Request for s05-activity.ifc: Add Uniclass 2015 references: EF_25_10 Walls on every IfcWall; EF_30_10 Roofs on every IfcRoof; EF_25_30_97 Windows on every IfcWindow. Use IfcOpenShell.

First a look at what the model holds.

```python
import ifcopenshell

model = ifcopenshell.open("s05-activity.ifc")
print(model.schema)
print("classifications:", [c.Name for c in model.by_type("IfcClassification")])
for ifc_class in ("IfcDoor", "IfcRoof", "IfcStair", "IfcWall", "IfcWindow"):
    print(ifc_class, len(model.by_type(ifc_class)))
```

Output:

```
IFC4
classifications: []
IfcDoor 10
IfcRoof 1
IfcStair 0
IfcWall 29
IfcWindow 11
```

```python
import ifcopenshell
import ifcopenshell.api.classification

model = ifcopenshell.open("s05-activity.ifc")

system = ifcopenshell.api.classification.add_classification(model, classification="Uniclass 2015")

codes = {
    "IfcWall": ("EF_25_10", "Walls"),
    "IfcRoof": ("EF_30_10", "Roofs"),
    "IfcWindow": ("EF_25_30_97", "Windows"),
}
for ifc_class, (code, name) in codes.items():
    products = model.by_type(ifc_class)
    ifcopenshell.api.classification.add_reference(
        model, products=products, classification=system, identification=code, name=name
    )
    print(code, len(products))

model.write("s05-activity_v2.ifc")
```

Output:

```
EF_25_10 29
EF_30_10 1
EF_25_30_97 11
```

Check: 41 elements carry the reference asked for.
